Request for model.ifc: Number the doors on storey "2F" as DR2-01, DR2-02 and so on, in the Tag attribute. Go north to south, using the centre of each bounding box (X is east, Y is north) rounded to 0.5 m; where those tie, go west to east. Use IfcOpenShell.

First a look at what the model holds.

```python
import ifcopenshell
import ifcopenshell.util.element
import ifcopenshell.util.placement

model = ifcopenshell.open("model.ifc")
print(model.schema)
storey = next(s for s in model.by_type("IfcBuildingStorey") if s.Name == "2F")
doors = [e for e in ifcopenshell.util.element.get_decomposition(storey) if e.is_a("IfcDoor")]
for e in sorted(doors, key=lambda e: e.id()):
    origin = ifcopenshell.util.placement.get_local_placement(e.ObjectPlacement)[:3, 3]
    print(e.id(), e.Tag, e.Name, origin.round(2) + 0.0, sep=" | ")
```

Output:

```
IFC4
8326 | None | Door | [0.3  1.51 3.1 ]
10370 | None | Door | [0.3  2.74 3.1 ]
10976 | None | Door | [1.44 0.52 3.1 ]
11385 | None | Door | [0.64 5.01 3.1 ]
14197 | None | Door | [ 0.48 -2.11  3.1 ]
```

```python
import ifcopenshell
import ifcopenshell.geom
import ifcopenshell.util.element
import ifcopenshell.util.shape

model = ifcopenshell.open("model.ifc")
settings = ifcopenshell.geom.settings()
settings.set("use-world-coords", True)


def centre(element):
    shape = ifcopenshell.geom.create_shape(settings, element)
    return ifcopenshell.util.shape.get_bbox_centroid(shape.geometry)


storey = next(s for s in model.by_type("IfcBuildingStorey") if s.Name == "2F")
doors = [e for e in ifcopenshell.util.element.get_decomposition(storey) if e.is_a("IfcDoor")]

# Insertion points can sit at a corner or the storey origin, so sort by the geometry (in metres).
centres = {e: centre(e) for e in doors}
doors.sort(key=lambda e: (-round(centres[e][1] / 0.5), centres[e][0]))

for i, e in enumerate(doors, start=1):
    number = f"DR2-{i:02d}"
    e.Tag = number
    print(e.id(), number)

model.write("model_updated.ifc")
```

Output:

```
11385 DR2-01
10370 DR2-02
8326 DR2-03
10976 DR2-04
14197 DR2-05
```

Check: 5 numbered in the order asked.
